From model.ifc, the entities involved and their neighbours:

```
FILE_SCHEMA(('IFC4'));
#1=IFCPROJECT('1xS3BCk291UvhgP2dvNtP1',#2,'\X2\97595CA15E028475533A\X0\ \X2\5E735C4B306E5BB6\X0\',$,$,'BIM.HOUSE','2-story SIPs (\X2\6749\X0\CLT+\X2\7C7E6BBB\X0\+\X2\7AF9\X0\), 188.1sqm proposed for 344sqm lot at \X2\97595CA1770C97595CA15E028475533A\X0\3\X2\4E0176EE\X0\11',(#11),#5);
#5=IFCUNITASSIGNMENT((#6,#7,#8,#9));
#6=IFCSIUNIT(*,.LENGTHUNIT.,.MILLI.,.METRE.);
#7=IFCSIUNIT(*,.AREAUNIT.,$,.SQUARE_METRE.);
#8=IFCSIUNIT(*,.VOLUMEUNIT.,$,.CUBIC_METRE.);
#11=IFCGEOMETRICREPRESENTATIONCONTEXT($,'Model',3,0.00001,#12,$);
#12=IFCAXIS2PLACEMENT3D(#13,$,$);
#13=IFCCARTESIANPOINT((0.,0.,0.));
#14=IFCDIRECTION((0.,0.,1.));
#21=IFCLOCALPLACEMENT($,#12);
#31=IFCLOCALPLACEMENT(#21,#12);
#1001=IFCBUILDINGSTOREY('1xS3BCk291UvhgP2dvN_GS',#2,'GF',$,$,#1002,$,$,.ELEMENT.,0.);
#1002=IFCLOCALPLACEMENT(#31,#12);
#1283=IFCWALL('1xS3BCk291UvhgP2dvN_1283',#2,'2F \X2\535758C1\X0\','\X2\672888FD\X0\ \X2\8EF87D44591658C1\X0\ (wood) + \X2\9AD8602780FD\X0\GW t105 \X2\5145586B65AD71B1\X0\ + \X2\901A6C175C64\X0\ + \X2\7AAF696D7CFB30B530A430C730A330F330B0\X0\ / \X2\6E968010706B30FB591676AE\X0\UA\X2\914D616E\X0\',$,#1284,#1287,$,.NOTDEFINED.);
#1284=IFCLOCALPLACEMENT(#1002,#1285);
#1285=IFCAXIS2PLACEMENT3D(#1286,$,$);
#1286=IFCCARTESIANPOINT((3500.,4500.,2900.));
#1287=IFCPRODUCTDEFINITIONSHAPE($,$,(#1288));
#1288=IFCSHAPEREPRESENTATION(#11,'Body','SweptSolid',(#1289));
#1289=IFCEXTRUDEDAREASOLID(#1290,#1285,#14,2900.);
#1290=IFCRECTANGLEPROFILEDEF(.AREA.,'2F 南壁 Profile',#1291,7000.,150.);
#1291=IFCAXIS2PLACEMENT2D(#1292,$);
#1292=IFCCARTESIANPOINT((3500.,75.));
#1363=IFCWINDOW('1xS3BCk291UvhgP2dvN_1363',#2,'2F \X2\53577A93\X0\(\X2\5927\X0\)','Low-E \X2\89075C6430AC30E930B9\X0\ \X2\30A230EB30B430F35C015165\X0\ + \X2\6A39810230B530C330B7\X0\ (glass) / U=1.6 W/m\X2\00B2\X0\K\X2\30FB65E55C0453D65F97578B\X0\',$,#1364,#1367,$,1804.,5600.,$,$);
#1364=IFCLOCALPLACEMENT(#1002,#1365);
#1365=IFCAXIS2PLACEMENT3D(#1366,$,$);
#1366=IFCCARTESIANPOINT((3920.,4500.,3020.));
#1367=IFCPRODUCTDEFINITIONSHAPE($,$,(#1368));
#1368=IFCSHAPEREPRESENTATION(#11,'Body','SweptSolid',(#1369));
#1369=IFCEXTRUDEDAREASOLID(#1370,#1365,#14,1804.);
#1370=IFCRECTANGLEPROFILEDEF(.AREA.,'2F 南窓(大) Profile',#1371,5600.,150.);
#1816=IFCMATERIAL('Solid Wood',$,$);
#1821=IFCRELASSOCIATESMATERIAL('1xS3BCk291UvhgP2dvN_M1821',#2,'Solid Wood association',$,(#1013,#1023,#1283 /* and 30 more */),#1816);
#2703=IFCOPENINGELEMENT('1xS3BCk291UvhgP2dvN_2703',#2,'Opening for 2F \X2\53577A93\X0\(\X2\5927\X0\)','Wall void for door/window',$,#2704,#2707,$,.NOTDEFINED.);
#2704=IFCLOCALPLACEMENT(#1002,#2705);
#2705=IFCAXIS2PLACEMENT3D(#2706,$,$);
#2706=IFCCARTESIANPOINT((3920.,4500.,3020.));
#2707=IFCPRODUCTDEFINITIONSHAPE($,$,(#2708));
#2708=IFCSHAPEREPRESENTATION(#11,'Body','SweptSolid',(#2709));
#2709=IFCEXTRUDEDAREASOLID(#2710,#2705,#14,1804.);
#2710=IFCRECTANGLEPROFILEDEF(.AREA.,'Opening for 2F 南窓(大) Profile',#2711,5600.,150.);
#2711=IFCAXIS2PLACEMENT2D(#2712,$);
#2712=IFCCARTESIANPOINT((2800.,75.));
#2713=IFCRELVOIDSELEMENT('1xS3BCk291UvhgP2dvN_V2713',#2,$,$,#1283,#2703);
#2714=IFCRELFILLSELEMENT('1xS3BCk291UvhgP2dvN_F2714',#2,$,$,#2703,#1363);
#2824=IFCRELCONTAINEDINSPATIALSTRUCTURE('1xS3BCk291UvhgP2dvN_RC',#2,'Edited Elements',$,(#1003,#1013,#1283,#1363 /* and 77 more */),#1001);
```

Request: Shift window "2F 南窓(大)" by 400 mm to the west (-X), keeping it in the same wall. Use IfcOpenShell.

```python
import ifcopenshell
import ifcopenshell.api.geometry
import ifcopenshell.util.placement
import ifcopenshell.util.unit

model = ifcopenshell.open("model.ifc")
unit_scale = ifcopenshell.util.unit.calculate_unit_scale(model)

window = model.by_guid("1xS3BCk291UvhgP2dvN_1363")
opening = window.FillsVoids[0].RelatingOpeningElement
wall = opening.VoidsElements[0].RelatingBuildingElement

wall_matrix = ifcopenshell.util.placement.get_local_placement(wall.ObjectPlacement)
shift = wall_matrix[:3, 0] * -0.4 / unit_scale
before = ifcopenshell.util.placement.get_local_placement(window.ObjectPlacement)[:3, 3].copy()

# The window is not placed relative to its opening, so move both.
for product in (opening, window):
    matrix = ifcopenshell.util.placement.get_local_placement(product.ObjectPlacement)
    matrix[:3, 3] += shift
    ifcopenshell.api.geometry.edit_object_placement(model, product=product, matrix=matrix, is_si=False)

after = ifcopenshell.util.placement.get_local_placement(window.ObjectPlacement)[:3, 3]
print("window moved by", (after - before).round(3) + 0.0)

model.write("model-out.ifc")
```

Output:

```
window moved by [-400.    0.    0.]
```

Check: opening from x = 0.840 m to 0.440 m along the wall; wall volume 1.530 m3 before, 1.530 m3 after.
